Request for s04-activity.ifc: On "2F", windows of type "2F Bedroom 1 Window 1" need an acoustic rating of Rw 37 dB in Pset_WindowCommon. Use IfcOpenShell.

First a look at what the model holds.

```python
import ifcopenshell
import ifcopenshell.util.element

model = ifcopenshell.open("s04-activity.ifc")
print(model.schema)
storey = next(s for s in model.by_type("IfcBuildingStorey") if s.Name == "2F")
windows = [e for e in ifcopenshell.util.element.get_decomposition(storey) if e.is_a("IfcWindow")]
seen = {}
for e in windows:
    element_type = ifcopenshell.util.element.get_type(e)
    key = (element_type.Name if element_type != e and element_type else None, ifcopenshell.util.element.get_pset(e, "Pset_WindowCommon", "AcousticRating"))
    seen[key] = seen.get(key, 0) + 1
for (name, value), count in sorted(seen.items(), key=str):
    print(count, "x", name, "|", value)
```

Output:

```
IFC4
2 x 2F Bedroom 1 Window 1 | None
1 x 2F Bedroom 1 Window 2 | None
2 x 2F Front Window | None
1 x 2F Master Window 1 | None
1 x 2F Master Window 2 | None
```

```python
import ifcopenshell
import ifcopenshell.api.pset
import ifcopenshell.util.element

model = ifcopenshell.open("s04-activity.ifc")

storey = next(s for s in model.by_type("IfcBuildingStorey") if s.Name == "2F")
windows = [e for e in ifcopenshell.util.element.get_decomposition(storey) if e.is_a("IfcWindow")]

count = 0
for e in windows:
    element_type = ifcopenshell.util.element.get_type(e)
    if element_type in (None, e) or element_type.Name != "2F Bedroom 1 Window 1":
        continue
    # add_pset returns the element's existing set when there is one.
    pset = ifcopenshell.api.pset.add_pset(model, product=e, name="Pset_WindowCommon")
    ifcopenshell.api.pset.edit_pset(model, pset=pset, properties={"AcousticRating": "Rw 37 dB"})
    count += 1

print(count, "windows updated")

model.write("s04-activity_updated.ifc")
```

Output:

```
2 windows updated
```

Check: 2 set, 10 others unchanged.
